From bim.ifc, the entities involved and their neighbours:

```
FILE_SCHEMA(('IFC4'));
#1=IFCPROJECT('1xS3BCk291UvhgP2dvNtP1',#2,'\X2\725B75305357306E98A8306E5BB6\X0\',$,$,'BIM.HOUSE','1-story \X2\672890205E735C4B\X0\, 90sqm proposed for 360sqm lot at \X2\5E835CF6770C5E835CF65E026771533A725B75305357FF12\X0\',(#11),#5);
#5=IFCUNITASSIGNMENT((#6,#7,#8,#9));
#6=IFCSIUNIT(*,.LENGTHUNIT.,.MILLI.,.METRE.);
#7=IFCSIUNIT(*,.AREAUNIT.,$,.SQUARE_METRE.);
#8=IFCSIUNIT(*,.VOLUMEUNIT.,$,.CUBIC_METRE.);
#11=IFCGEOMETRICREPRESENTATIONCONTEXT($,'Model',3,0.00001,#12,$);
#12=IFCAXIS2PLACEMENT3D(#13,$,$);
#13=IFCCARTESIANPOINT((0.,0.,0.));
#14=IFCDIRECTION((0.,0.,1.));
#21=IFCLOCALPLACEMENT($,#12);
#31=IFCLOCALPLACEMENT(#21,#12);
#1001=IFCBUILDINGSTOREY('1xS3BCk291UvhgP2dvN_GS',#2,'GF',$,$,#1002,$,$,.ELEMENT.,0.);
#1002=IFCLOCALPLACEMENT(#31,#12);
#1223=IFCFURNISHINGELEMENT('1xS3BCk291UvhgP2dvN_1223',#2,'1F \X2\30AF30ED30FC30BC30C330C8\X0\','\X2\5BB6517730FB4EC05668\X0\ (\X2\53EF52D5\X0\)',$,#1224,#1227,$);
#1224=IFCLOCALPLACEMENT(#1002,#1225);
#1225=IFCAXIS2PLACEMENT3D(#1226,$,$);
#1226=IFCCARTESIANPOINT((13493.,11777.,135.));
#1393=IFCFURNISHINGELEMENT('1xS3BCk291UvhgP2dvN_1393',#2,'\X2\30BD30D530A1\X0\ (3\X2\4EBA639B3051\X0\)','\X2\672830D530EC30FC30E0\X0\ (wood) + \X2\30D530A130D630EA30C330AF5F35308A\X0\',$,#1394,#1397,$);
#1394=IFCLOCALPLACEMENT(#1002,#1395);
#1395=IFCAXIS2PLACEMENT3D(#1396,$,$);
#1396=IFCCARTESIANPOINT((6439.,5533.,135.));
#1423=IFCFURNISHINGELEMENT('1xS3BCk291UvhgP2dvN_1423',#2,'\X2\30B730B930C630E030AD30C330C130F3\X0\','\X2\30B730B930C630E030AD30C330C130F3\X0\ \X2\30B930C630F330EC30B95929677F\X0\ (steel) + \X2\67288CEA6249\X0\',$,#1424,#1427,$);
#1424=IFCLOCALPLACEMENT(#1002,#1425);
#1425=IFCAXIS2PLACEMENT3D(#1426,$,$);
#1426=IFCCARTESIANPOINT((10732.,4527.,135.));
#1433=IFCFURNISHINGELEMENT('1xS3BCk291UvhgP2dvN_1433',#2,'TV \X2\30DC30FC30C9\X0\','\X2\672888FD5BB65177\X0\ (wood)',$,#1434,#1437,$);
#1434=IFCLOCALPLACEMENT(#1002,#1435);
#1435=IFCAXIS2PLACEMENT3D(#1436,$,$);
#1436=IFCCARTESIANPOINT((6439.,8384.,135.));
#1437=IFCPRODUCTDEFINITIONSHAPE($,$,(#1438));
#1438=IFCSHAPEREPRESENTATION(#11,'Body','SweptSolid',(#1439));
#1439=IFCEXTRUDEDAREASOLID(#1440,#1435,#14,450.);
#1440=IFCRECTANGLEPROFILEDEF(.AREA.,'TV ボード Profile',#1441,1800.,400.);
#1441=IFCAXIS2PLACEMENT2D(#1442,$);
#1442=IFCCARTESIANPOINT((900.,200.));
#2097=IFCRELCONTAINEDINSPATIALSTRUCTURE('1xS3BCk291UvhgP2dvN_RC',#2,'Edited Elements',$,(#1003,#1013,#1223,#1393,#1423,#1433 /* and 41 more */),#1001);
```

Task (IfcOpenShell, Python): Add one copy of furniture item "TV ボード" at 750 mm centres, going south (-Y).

```python
import numpy as np
import ifcopenshell
import ifcopenshell.api.geometry
import ifcopenshell.api.root
import ifcopenshell.util.element
import ifcopenshell.util.placement
import ifcopenshell.util.unit

model = ifcopenshell.open("bim.ifc")
unit_scale = ifcopenshell.util.unit.calculate_unit_scale(model)


def reuse_history(source, copy):
    """copy_class also copies each property set's owner history, people and application; keep the originals."""
    for rel in copy.IsDefinedBy:
        if rel.is_a("IfcRelDefinesByProperties") and (history := rel.RelatingPropertyDefinition.OwnerHistory):
            rel.RelatingPropertyDefinition.OwnerHistory = source.OwnerHistory
            ifcopenshell.util.element.remove_deep2(model, history)


source = model.by_guid("1xS3BCk291UvhgP2dvN_1433")
base = ifcopenshell.util.placement.get_local_placement(source.ObjectPlacement)
step = np.array([0.0, -1.0, 0.0]) * 0.75 / unit_scale

for i in range(1, 2):
    copy = ifcopenshell.api.root.copy_class(model, product=source)
    copy.Representation = ifcopenshell.util.element.copy_deep(
        model, source.Representation, exclude=["IfcGeometricRepresentationContext", "IfcRepresentationMap"]
    )
    reuse_history(source, copy)
    matrix = base.copy()
    matrix[:3, 3] += i * step
    print("added at", matrix[:3, 3].round(3) + 0.0)
    ifcopenshell.api.geometry.edit_object_placement(model, product=copy, matrix=matrix, is_si=False)

model.write("bim_rev.ifc")
```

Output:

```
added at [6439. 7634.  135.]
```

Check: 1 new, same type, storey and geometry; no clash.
